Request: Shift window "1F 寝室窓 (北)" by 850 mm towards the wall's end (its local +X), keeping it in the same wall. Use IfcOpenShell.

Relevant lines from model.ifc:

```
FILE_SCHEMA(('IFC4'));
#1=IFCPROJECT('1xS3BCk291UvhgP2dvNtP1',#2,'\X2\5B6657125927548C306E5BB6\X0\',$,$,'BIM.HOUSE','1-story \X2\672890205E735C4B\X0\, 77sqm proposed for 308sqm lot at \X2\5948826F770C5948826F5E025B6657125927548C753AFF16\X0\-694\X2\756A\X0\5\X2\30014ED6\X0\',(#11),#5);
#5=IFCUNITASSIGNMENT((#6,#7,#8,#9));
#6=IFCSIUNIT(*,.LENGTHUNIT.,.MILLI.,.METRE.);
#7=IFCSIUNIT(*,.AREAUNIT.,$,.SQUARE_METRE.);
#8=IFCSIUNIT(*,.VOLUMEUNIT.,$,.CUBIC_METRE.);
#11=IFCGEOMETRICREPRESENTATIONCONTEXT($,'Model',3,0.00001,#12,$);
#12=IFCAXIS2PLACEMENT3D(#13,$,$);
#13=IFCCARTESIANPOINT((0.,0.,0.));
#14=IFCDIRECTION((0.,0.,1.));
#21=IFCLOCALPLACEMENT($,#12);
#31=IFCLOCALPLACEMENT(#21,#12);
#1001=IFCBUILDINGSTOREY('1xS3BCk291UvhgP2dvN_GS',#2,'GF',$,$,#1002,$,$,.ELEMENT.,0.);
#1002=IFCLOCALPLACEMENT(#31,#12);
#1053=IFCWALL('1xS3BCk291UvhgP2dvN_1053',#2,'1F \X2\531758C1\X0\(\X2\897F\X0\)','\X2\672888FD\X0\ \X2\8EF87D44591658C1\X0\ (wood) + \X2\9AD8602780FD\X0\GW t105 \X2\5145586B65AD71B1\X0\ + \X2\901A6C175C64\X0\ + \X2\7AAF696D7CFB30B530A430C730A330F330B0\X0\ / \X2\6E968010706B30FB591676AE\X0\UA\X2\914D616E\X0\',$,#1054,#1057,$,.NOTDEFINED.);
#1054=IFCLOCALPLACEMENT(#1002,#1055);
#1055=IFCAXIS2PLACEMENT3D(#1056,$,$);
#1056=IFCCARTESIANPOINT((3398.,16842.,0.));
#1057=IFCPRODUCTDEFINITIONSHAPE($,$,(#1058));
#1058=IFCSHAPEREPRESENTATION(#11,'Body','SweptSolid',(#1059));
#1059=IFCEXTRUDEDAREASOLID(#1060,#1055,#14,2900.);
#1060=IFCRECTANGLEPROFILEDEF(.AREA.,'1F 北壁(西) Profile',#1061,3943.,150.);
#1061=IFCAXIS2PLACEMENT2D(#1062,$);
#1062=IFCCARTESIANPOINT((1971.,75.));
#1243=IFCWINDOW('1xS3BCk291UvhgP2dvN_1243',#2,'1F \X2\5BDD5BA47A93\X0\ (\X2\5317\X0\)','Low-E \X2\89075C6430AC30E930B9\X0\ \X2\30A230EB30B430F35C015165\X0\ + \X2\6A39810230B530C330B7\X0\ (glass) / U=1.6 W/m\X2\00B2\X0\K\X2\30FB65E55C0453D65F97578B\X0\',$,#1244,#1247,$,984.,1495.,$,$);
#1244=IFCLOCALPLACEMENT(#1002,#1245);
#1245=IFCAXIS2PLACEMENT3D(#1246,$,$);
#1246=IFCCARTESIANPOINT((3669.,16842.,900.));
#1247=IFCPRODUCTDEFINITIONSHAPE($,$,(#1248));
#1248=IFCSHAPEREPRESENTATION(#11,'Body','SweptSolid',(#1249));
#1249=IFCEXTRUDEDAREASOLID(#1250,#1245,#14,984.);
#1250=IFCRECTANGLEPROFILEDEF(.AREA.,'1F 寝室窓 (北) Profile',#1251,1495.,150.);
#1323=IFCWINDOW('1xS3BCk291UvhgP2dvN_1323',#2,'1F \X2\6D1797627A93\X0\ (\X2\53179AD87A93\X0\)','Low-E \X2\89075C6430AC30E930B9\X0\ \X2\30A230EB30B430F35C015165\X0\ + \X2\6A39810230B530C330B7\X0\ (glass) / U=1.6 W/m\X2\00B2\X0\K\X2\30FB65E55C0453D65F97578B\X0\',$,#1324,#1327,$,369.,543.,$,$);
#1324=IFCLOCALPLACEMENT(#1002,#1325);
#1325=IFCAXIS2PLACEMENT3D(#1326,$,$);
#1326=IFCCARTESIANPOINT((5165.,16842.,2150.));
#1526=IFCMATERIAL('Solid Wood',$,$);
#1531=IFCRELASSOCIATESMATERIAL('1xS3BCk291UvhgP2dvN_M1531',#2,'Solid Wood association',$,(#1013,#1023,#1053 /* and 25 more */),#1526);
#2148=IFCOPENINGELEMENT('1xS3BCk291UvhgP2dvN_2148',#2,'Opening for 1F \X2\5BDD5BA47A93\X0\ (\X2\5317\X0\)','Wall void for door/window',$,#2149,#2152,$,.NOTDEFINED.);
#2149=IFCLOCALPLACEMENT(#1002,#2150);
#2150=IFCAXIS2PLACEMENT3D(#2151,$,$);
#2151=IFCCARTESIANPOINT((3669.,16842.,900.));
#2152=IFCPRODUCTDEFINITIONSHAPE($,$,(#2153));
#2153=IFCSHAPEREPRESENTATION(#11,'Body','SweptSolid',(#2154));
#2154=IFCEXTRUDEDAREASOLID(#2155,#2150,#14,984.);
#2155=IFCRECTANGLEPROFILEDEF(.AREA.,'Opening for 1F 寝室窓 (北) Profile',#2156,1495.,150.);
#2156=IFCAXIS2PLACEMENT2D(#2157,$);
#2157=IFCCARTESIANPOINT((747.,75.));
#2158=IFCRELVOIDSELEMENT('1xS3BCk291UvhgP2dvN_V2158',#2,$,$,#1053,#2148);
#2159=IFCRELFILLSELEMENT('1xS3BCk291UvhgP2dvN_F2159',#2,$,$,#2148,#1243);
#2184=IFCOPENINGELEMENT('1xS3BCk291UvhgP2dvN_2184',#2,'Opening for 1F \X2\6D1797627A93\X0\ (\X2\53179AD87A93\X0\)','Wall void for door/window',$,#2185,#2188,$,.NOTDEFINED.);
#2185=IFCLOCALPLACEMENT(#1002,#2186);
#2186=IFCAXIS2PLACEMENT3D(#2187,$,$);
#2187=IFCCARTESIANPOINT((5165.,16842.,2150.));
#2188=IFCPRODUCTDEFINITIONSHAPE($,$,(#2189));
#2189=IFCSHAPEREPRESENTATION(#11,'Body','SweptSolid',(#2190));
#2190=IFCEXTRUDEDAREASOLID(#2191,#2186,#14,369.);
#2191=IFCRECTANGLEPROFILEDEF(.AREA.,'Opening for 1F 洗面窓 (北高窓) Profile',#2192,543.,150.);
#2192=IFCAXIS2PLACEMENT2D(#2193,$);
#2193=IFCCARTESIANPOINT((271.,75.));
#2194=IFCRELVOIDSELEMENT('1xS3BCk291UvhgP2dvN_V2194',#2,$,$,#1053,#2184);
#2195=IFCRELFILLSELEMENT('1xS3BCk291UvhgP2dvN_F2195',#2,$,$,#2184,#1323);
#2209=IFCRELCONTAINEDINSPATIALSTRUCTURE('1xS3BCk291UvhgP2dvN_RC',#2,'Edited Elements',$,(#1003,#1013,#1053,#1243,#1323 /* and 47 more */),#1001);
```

```python
import ifcopenshell
import ifcopenshell.api.geometry
import ifcopenshell.util.placement
import ifcopenshell.util.unit

model = ifcopenshell.open("model.ifc")
unit_scale = ifcopenshell.util.unit.calculate_unit_scale(model)

window = model.by_guid("1xS3BCk291UvhgP2dvN_1243")
opening = window.FillsVoids[0].RelatingOpeningElement
wall = opening.VoidsElements[0].RelatingBuildingElement

wall_matrix = ifcopenshell.util.placement.get_local_placement(wall.ObjectPlacement)
shift = wall_matrix[:3, 0] * 0.85 / unit_scale
before = ifcopenshell.util.placement.get_local_placement(window.ObjectPlacement)[:3, 3].copy()

# The window is not placed relative to its opening, so move both.
for product in (opening, window):
    matrix = ifcopenshell.util.placement.get_local_placement(product.ObjectPlacement)
    matrix[:3, 3] += shift
    ifcopenshell.api.geometry.edit_object_placement(model, product=product, matrix=matrix, is_si=False)

after = ifcopenshell.util.placement.get_local_placement(window.ObjectPlacement)[:3, 3]
print("window moved by", (after - before).round(3) + 0.0)

model.write("model-out.ifc")
```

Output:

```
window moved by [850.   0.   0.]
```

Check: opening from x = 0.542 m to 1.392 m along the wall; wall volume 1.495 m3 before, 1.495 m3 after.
